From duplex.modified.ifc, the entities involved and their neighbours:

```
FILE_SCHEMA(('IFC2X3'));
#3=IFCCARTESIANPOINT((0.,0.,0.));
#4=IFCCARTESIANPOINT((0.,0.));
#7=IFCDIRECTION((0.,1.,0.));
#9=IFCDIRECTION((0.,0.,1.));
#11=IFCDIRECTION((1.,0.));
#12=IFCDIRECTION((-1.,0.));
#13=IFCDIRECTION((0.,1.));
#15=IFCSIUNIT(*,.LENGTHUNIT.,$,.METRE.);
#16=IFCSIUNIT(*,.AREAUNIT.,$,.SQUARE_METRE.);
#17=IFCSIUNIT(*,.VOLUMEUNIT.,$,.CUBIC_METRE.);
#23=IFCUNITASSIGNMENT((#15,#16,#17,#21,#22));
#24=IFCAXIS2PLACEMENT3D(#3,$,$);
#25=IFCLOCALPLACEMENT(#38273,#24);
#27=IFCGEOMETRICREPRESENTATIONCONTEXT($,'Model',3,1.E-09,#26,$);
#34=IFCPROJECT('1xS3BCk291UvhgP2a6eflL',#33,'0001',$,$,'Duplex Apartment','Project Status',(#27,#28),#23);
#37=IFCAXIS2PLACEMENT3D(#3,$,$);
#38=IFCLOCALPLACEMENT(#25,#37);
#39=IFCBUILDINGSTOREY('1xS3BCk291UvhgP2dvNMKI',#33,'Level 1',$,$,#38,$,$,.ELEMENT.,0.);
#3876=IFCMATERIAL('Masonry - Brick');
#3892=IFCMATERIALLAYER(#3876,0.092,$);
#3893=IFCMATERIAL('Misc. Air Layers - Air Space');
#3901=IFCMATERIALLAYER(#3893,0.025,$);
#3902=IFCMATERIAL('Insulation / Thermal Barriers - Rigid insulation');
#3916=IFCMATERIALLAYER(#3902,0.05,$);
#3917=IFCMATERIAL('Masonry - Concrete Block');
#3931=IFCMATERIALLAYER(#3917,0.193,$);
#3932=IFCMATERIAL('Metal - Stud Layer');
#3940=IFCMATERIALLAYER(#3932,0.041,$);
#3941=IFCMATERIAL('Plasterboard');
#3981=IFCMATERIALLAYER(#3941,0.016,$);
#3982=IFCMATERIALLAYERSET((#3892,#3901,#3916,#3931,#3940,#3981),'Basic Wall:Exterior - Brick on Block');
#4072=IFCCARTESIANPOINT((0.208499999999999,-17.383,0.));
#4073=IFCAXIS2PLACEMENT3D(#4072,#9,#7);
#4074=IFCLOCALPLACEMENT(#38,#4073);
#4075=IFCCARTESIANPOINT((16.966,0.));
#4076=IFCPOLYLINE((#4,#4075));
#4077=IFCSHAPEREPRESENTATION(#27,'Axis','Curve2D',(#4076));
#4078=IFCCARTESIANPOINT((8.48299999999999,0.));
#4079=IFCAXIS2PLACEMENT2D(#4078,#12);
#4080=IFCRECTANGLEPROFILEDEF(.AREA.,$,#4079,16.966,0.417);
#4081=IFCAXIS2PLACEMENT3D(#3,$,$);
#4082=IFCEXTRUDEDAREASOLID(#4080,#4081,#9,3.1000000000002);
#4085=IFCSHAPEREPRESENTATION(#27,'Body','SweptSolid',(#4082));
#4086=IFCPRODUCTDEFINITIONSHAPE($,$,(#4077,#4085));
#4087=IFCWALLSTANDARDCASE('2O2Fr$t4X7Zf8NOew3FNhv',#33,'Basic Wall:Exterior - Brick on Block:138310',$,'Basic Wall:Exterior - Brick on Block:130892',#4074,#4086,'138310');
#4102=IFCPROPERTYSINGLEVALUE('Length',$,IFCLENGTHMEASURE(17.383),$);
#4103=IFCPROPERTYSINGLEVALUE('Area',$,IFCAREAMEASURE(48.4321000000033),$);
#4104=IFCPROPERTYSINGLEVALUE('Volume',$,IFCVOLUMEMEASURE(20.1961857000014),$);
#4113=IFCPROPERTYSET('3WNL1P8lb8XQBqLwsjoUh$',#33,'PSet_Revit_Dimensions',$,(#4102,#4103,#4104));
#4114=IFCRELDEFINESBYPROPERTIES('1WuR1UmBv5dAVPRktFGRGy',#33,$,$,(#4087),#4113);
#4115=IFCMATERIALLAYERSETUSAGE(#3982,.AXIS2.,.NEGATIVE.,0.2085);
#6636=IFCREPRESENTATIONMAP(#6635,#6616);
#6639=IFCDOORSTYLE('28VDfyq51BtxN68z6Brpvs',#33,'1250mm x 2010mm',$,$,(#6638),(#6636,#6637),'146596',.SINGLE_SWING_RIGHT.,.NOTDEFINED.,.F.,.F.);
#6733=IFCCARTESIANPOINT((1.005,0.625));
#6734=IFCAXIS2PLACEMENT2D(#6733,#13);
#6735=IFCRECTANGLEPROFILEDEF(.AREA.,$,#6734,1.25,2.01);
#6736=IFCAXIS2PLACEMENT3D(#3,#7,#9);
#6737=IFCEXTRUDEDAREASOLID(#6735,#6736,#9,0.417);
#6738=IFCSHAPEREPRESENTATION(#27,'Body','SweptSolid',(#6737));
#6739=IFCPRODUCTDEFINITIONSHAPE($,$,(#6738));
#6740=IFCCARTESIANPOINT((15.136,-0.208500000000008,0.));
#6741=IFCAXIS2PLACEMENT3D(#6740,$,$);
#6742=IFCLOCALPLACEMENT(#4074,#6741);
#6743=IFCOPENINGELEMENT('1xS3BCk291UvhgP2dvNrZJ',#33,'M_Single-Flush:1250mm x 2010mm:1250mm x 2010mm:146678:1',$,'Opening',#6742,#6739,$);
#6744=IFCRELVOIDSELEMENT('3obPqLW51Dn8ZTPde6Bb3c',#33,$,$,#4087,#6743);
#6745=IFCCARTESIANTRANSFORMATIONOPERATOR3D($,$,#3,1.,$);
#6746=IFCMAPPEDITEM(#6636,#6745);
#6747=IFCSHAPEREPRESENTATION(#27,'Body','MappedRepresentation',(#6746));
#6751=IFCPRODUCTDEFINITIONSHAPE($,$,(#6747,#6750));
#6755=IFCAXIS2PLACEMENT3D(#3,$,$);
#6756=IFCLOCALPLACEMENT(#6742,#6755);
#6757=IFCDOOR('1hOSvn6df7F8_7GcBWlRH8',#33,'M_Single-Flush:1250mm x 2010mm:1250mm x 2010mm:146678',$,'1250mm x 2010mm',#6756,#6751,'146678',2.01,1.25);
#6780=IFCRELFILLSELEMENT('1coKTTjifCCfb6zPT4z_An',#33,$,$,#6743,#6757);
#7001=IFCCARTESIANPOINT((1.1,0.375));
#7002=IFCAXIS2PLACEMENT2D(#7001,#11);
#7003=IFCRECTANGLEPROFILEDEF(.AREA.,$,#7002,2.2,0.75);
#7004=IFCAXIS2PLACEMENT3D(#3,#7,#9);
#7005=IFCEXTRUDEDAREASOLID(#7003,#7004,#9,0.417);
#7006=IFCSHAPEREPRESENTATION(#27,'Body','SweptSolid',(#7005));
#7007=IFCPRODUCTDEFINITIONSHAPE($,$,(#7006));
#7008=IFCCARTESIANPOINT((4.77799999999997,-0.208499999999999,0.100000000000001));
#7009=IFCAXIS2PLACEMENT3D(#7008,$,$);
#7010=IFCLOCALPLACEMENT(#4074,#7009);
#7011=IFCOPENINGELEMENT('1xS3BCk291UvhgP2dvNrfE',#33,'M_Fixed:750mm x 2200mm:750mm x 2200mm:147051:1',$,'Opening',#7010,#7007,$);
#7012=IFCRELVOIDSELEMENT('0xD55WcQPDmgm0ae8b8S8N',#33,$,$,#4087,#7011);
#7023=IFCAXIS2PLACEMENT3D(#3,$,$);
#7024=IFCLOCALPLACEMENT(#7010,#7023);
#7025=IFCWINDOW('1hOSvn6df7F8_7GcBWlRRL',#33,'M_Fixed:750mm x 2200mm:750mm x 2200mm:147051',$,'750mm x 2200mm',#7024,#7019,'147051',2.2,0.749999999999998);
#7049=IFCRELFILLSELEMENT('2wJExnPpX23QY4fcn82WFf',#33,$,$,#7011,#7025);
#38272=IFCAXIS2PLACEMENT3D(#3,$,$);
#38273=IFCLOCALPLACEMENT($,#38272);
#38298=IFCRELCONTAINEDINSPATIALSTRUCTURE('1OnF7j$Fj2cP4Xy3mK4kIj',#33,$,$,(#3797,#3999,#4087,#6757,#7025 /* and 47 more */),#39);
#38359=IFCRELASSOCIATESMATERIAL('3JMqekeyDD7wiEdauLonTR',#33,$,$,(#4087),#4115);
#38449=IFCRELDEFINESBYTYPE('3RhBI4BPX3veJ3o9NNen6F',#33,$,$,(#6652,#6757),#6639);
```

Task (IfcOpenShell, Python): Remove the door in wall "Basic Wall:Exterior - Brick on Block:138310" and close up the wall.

```python
import ifcopenshell
import ifcopenshell.api.feature
import ifcopenshell.api.pset
import ifcopenshell.api.root
import ifcopenshell.geom
import ifcopenshell.util.element
import ifcopenshell.util.shape
import ifcopenshell.util.unit

model = ifcopenshell.open("duplex.modified.ifc")
area_scale = ifcopenshell.util.unit.calculate_unit_scale(model, "AREAUNIT")
volume_scale = ifcopenshell.util.unit.calculate_unit_scale(model, "VOLUMEUNIT")
settings = ifcopenshell.geom.settings()


def volume(element):
    """Net volume in cubic metres, openings subtracted."""
    shape = ifcopenshell.geom.create_shape(settings, element)
    return ifcopenshell.util.shape.get_volume(shape.geometry)


door = model.by_guid("1hOSvn6df7F8_7GcBWlRH8")
opening = door.FillsVoids[0].RelatingOpeningElement
wall = opening.VoidsElements[0].RelatingBuildingElement
before = volume(wall)

ifcopenshell.api.root.remove_product(model, product=door)
ifcopenshell.api.feature.remove_feature(model, feature=opening)

after = volume(wall)
thickness = 0.417  # wall thickness in metres

# Update the wall's stored quantities.
pset = model.by_id(ifcopenshell.util.element.get_pset(wall, "PSet_Revit_Dimensions", should_inherit=False)["id"])
ifcopenshell.api.pset.edit_pset(model, pset=pset, properties={
    "Area": model.create_entity("IfcAreaMeasure", after / thickness / area_scale),
    "Volume": model.create_entity("IfcVolumeMeasure", after / volume_scale),
})

print(f"wall volume {before:.3f} -> {after:.3f} m3")

model.write("duplex.modified-out.ifc")
```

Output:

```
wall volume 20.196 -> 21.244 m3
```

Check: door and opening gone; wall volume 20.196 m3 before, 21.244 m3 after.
